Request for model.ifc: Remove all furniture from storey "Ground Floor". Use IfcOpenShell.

First a look at what the model holds.

```python
import ifcopenshell
import ifcopenshell.util.element

model = ifcopenshell.open("model.ifc")
print(model.schema)
storey = next(s for s in model.by_type("IfcBuildingStorey") if s.Name == "Ground Floor")
furniture = [e for e in ifcopenshell.util.element.get_decomposition(storey) if e.is_a("IfcFurnishingElement")]
seen = {}
for e in furniture:
    element_type = ifcopenshell.util.element.get_type(e)
    name = element_type.Name if element_type not in (None, e) else None
    seen[name] = seen.get(name, 0) + 1
for name, count in sorted(seen.items(), key=str):
    print(count, "x", name)
```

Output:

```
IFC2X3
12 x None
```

```python
import ifcopenshell
import ifcopenshell.api.root
import ifcopenshell.util.element

model = ifcopenshell.open("model.ifc")

storey = next(s for s in model.by_type("IfcBuildingStorey") if s.Name == "Ground Floor")
furniture = [e for e in ifcopenshell.util.element.get_decomposition(storey) if e.is_a("IfcFurnishingElement")]

for e in furniture:
    ifcopenshell.api.root.remove_product(model, product=e)
print(len(furniture), "removed")

model.write("model_v2.ifc")
```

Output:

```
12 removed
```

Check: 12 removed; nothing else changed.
